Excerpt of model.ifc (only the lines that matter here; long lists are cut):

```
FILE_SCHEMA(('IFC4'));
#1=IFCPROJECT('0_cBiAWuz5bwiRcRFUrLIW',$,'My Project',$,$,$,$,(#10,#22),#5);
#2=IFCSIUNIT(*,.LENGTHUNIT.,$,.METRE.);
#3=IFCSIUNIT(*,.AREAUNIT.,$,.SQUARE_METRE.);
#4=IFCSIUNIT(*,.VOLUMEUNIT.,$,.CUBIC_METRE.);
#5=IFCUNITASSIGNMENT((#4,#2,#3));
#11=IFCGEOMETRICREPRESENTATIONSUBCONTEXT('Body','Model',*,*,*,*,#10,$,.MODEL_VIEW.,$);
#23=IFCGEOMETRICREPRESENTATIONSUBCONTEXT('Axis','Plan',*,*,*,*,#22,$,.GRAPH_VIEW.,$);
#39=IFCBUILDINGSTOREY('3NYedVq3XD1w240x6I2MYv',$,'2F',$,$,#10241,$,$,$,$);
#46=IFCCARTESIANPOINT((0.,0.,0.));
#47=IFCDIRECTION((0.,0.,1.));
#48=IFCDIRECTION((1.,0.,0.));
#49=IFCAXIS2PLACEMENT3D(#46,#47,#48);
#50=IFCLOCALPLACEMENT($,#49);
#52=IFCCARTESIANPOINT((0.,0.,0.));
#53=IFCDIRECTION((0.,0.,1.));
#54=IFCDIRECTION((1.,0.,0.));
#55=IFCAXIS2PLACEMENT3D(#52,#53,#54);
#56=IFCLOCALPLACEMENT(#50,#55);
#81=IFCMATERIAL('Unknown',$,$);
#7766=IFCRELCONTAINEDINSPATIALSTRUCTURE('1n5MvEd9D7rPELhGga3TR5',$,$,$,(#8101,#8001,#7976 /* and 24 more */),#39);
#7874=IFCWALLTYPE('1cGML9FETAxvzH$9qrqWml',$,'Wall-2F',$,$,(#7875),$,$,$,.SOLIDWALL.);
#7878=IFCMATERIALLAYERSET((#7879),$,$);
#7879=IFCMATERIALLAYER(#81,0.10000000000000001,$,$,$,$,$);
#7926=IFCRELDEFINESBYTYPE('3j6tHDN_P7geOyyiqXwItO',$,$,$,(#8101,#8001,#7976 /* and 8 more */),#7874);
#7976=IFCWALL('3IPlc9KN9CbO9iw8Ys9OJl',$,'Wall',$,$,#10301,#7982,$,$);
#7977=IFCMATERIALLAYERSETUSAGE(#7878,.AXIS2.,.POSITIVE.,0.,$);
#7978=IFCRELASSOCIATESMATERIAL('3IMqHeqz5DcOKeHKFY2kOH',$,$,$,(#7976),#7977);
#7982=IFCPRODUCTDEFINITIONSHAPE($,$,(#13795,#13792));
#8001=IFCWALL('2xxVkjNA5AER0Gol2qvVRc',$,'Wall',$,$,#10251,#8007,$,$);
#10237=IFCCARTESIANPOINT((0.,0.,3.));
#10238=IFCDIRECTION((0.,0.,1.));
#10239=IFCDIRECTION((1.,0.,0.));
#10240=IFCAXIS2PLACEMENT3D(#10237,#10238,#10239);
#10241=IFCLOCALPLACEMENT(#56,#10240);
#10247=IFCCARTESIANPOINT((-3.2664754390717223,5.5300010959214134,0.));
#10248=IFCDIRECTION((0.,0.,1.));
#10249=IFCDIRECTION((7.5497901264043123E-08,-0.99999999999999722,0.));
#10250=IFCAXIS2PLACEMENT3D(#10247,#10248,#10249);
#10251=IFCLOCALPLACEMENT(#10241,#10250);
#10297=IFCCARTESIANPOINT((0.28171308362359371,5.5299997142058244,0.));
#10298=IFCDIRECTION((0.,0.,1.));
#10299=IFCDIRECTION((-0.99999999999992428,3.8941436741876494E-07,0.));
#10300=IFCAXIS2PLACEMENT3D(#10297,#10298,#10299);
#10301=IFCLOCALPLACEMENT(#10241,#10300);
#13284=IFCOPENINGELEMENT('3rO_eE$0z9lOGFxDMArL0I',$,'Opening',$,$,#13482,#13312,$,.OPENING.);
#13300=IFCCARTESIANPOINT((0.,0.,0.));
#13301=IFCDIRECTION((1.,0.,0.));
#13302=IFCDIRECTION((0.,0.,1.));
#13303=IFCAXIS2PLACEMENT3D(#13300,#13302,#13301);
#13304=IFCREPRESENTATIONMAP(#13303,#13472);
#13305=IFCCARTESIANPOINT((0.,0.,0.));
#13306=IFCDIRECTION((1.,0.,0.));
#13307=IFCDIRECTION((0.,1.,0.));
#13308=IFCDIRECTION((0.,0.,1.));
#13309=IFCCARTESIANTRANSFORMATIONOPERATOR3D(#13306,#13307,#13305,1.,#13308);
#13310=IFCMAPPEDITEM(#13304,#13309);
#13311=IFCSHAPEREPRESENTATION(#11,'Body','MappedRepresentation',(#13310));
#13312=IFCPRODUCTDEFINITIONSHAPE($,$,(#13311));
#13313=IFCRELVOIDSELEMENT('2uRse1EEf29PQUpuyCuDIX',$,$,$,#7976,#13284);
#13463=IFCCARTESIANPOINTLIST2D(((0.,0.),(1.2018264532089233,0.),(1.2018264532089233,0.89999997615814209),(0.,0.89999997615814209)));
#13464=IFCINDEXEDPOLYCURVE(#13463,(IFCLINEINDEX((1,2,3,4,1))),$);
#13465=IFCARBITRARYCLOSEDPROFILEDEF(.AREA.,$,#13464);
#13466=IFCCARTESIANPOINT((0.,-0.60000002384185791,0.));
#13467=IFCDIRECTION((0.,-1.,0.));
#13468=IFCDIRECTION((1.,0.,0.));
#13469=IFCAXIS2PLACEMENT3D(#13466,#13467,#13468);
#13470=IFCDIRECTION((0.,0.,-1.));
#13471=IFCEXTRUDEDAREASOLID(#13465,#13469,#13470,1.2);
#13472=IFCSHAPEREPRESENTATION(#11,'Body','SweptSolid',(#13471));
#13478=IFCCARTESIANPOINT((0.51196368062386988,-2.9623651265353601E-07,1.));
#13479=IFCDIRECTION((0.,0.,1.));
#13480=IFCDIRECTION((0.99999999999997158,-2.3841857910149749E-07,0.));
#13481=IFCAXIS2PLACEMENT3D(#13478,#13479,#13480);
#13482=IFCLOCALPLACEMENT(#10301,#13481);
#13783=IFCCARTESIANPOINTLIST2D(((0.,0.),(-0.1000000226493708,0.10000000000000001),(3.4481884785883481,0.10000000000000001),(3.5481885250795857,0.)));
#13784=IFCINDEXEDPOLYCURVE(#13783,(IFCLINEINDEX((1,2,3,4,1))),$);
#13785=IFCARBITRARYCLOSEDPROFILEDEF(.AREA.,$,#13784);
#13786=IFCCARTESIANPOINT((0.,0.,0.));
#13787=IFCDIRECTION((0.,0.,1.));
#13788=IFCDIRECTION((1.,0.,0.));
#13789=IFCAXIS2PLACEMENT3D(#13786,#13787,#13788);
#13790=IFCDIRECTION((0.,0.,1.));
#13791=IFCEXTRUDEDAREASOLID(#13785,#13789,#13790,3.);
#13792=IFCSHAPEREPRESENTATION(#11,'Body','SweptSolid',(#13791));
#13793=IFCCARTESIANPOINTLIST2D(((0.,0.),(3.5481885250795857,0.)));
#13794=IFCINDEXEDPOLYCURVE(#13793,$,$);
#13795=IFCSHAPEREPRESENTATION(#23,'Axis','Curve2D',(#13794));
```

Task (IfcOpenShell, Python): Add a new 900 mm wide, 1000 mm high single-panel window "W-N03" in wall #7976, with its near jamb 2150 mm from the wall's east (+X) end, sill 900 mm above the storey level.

```python
import numpy as np
import ifcopenshell
import ifcopenshell.api.feature
import ifcopenshell.api.geometry
import ifcopenshell.api.root
import ifcopenshell.api.spatial
import ifcopenshell.geom
import ifcopenshell.util.element
import ifcopenshell.util.placement
import ifcopenshell.util.representation
import ifcopenshell.util.shape
import ifcopenshell.util.unit

model = ifcopenshell.open("model.ifc")
unit_scale = ifcopenshell.util.unit.calculate_unit_scale(model)
settings = ifcopenshell.geom.settings()


def volume(element):
    """Net volume in cubic metres, openings subtracted."""
    shape = ifcopenshell.geom.create_shape(settings, element)
    return ifcopenshell.util.shape.get_volume(shape.geometry)


wall = model.by_id(7976)
storey = ifcopenshell.util.element.get_container(wall, ifc_class="IfcBuildingStorey")
context = ifcopenshell.util.representation.get_context(model, "Model", "Body", "MODEL_VIEW")
before = volume(wall)

width, height, from_end, sill = 0.9, 1, 2.15, 0.9  # metres

# The wall runs along its own X axis, and the end named is its -X end.
wall_shape = ifcopenshell.geom.create_shape(settings, wall)
x, y, z = ifcopenshell.util.shape.get_vertices(wall_shape.geometry).T
start = x.min() + from_end
face, thickness = float(y.min()), float(y.max() - y.min())
wall_matrix = ifcopenshell.util.placement.get_local_placement(wall.ObjectPlacement)
level = ifcopenshell.util.placement.get_local_placement(storey.ObjectPlacement)[2, 3]


def in_wall(x, y):
    """Placement at x, y metres in the wall's axes, at sill height."""
    matrix = wall_matrix.copy()
    matrix[:, 3] = wall_matrix @ np.array([x / unit_scale, y / unit_scale, 0.0, 1.0])
    matrix[2, 3] = level + sill / unit_scale
    return matrix


# Opening: a box that overshoots both wall faces by 50 mm.
opening = ifcopenshell.api.root.create_entity(model, ifc_class="IfcOpeningElement", predefined_type="OPENING")
box = ifcopenshell.api.geometry.add_wall_representation(
    model, context=context, length=width, height=height, thickness=thickness + 0.1
)
ifcopenshell.api.geometry.assign_representation(model, product=opening, representation=box)
ifcopenshell.api.geometry.edit_object_placement(model, product=opening, matrix=in_wall(start, face - 0.05), is_si=False)
ifcopenshell.api.feature.add_feature(model, feature=opening, element=wall)

window = ifcopenshell.api.root.create_entity(model, ifc_class="IfcWindow", name="W-N03", predefined_type="WINDOW")
window.OverallWidth, window.OverallHeight = width / unit_scale, height / unit_scale
window.PartitioningType = "SINGLE_PANEL"
body = ifcopenshell.api.geometry.add_window_representation(
    model,
    context=context,
    overall_width=window.OverallWidth,
    overall_height=window.OverallHeight,
    partition_type="SINGLE_PANEL",
)
ifcopenshell.api.geometry.assign_representation(model, product=window, representation=body)
ifcopenshell.api.spatial.assign_container(model, products=[window], relating_structure=storey)
ifcopenshell.api.feature.add_filling(model, opening=opening, element=window)

# Centre the window in the wall's thickness.
ifcopenshell.api.geometry.edit_object_placement(model, product=window, matrix=in_wall(start, face), is_si=False)
window_shape = ifcopenshell.geom.create_shape(settings, window)
depth = ifcopenshell.util.shape.get_vertices(window_shape.geometry)[:, 1]
offset = face + thickness / 2 - (depth.min() + depth.max()) / 2
ifcopenshell.api.geometry.edit_object_placement(model, product=window, matrix=in_wall(start, offset), is_si=False)

after = volume(wall)

print(f"wall volume {before:.3f} -> {after:.3f} m3")

model.write("model_updated.ifc")
```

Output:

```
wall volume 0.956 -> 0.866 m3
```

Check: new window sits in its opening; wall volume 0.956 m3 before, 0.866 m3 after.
